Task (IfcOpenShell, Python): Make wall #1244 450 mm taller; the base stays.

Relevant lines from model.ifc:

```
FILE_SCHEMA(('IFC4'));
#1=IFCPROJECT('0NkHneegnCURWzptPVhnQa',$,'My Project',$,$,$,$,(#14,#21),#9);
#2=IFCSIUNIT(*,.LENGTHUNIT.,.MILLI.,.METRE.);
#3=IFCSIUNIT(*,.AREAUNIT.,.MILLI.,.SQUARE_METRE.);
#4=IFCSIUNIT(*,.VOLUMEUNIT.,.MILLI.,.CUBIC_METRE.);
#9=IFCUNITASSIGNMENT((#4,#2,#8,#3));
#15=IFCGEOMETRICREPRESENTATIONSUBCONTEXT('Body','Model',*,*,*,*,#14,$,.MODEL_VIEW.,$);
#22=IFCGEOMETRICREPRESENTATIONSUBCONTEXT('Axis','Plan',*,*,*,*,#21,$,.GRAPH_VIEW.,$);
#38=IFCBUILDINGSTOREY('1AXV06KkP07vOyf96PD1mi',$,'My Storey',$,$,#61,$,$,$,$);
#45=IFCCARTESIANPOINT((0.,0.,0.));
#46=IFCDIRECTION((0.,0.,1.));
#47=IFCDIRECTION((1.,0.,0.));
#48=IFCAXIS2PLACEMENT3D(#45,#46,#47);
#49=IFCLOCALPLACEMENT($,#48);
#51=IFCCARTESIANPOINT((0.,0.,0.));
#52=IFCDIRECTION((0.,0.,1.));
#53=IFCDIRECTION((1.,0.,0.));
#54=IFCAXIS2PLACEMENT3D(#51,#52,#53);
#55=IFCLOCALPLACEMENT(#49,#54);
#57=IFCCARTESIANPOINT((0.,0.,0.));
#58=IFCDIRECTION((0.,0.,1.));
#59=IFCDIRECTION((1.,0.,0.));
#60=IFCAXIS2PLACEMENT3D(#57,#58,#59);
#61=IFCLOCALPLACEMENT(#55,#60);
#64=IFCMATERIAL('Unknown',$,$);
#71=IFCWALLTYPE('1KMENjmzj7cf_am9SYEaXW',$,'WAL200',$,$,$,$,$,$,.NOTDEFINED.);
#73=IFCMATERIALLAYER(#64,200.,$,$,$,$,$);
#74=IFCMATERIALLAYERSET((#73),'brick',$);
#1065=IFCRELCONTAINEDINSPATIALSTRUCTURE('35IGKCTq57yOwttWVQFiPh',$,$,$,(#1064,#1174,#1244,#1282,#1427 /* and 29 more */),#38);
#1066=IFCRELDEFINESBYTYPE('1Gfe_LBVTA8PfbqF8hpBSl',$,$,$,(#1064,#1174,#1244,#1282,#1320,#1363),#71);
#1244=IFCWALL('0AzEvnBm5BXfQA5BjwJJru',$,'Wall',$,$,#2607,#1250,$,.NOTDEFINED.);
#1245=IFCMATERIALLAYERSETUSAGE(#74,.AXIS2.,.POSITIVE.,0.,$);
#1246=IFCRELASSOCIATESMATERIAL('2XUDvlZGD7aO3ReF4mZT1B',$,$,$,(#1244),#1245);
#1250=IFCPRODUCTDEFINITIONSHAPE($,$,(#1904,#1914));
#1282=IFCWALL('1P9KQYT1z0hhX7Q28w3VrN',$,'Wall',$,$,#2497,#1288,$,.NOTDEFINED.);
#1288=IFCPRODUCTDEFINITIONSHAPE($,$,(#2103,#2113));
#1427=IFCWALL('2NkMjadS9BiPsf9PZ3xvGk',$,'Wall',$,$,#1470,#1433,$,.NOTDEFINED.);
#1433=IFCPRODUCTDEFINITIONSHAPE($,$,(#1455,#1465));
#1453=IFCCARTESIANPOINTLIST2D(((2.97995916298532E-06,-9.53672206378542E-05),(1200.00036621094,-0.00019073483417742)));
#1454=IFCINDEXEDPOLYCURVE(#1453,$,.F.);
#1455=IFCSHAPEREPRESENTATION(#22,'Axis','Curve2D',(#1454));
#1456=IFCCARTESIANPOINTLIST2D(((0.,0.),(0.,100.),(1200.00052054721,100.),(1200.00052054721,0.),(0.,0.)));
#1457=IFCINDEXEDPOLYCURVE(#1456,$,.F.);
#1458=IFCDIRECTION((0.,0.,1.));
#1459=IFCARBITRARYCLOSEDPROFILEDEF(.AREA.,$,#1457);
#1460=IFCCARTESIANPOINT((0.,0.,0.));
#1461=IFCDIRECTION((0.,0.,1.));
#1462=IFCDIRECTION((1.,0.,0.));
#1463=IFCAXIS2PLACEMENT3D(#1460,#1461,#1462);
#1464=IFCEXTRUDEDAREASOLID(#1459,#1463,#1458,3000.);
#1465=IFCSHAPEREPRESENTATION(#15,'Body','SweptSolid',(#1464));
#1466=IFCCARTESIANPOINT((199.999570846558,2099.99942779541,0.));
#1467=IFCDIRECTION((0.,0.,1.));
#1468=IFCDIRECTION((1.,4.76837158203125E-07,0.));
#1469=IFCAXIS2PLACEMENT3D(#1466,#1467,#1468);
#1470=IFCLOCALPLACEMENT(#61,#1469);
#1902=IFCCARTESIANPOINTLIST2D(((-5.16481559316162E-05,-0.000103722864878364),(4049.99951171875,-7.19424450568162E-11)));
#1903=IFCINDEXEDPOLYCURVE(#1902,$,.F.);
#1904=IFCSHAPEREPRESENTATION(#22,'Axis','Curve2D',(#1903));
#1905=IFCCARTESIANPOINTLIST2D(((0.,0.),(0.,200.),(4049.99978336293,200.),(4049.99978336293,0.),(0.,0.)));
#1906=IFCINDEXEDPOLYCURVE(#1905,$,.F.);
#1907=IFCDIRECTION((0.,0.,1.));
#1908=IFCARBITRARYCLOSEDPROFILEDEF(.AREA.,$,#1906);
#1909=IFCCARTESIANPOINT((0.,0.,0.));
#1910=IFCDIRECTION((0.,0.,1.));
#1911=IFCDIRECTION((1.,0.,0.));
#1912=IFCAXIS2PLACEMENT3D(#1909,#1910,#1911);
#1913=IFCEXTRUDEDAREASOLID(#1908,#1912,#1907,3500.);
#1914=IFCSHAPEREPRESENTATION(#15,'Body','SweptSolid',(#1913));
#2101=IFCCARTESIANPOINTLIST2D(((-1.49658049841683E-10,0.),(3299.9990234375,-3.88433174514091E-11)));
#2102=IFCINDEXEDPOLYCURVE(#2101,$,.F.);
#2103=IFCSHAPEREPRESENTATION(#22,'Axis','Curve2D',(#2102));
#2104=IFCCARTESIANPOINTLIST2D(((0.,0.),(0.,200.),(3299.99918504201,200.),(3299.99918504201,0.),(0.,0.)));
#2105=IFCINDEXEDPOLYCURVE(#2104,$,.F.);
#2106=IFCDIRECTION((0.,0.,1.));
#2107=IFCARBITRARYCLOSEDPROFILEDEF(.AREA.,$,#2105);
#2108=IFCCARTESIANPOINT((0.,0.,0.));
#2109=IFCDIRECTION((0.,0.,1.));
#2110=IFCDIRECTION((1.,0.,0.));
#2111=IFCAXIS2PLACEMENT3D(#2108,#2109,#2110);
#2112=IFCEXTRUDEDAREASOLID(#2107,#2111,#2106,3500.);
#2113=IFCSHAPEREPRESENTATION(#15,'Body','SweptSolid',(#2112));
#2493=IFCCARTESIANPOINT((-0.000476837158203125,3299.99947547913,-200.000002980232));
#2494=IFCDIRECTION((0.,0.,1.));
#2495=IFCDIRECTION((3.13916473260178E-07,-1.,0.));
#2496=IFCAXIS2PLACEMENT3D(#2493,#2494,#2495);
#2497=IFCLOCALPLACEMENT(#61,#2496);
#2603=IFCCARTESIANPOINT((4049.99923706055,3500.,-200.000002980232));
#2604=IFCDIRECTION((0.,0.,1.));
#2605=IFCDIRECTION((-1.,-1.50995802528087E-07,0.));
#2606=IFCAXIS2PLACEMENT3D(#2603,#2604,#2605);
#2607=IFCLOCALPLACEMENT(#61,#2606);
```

```python
import ifcopenshell
import ifcopenshell.geom
import ifcopenshell.util.representation
import ifcopenshell.util.shape

model = ifcopenshell.open("model.ifc")
settings = ifcopenshell.geom.settings()


def volume(element):
    """Net volume in cubic metres, openings subtracted."""
    shape = ifcopenshell.geom.create_shape(settings, element)
    return ifcopenshell.util.shape.get_volume(shape.geometry)


wall = model.by_id(1244)
before = volume(wall)

body = ifcopenshell.util.representation.get_representation(wall, "Model", "Body")
solid = body.Items[0]
old_height = solid.Depth
solid.Depth += 450.0
after = volume(wall)

print(f"height {old_height:g} -> {solid.Depth:g}, volume {before:.3f} -> {after:.3f} m3")

model.write("model_edited.ifc")
```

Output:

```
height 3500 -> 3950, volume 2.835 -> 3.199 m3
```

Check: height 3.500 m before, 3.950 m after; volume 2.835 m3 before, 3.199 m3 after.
